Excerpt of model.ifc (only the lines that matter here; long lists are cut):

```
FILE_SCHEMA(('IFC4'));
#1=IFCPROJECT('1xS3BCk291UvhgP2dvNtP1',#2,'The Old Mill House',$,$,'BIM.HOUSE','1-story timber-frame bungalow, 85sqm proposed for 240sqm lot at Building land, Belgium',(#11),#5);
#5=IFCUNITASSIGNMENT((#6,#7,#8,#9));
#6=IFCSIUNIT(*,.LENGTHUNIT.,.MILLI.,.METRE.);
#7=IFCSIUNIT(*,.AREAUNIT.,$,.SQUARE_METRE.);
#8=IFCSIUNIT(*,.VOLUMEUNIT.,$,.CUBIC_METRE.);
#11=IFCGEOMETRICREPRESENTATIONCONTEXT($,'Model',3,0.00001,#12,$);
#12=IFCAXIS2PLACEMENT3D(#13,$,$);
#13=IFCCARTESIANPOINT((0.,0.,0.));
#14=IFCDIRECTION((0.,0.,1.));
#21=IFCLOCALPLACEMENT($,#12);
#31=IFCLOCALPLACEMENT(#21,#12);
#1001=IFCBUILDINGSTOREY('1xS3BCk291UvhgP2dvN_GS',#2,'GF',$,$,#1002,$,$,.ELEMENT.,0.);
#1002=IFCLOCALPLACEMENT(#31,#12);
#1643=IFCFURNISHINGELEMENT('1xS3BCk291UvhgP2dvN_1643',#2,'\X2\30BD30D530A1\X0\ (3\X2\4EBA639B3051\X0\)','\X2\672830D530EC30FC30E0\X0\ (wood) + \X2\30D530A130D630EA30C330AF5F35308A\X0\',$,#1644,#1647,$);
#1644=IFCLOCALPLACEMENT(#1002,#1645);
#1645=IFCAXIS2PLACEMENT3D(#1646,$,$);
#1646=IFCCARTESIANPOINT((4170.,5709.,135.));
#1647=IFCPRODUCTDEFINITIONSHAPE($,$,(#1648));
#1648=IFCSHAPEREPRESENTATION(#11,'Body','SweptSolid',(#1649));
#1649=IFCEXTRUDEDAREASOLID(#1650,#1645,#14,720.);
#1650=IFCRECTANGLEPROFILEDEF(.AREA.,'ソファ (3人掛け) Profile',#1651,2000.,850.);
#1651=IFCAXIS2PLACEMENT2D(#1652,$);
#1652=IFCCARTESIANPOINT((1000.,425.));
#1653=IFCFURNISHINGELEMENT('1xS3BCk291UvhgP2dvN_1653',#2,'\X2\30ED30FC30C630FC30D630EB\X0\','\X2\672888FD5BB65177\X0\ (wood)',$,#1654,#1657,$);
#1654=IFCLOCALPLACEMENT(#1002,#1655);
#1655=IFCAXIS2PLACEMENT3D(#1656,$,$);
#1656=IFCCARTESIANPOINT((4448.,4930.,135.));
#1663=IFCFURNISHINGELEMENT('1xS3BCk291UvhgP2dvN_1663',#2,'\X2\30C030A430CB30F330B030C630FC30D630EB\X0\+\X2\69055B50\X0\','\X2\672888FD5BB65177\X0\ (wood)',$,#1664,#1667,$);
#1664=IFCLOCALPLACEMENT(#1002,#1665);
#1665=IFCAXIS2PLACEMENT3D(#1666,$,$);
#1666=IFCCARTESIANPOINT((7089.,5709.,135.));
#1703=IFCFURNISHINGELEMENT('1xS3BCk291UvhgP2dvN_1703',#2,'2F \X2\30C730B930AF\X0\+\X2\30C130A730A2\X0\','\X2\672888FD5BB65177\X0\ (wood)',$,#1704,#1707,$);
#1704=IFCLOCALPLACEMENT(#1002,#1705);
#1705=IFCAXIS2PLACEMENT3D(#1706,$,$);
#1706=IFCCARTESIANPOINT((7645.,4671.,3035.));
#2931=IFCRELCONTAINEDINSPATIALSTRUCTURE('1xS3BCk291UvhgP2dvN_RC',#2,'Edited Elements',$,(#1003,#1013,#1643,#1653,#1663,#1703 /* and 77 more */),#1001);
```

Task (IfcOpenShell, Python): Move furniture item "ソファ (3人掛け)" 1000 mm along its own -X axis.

```python
import ifcopenshell
import ifcopenshell.api.geometry
import ifcopenshell.util.placement
import ifcopenshell.util.unit

model = ifcopenshell.open("model.ifc")
unit_scale = ifcopenshell.util.unit.calculate_unit_scale(model)

item = model.by_id(1643)
matrix = ifcopenshell.util.placement.get_local_placement(item.ObjectPlacement)
matrix[:3, 3] -= matrix[:3, 0] * 1 / unit_scale
ifcopenshell.api.geometry.edit_object_placement(model, product=item, matrix=matrix, is_si=False)

print(ifcopenshell.util.placement.get_local_placement(item.ObjectPlacement).round(3) + 0.0)

model.write("model_updated.ifc")
```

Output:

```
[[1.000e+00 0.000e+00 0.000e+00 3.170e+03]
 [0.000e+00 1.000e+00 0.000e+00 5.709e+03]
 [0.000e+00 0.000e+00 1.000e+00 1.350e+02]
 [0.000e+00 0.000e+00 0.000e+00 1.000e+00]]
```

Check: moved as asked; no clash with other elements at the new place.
